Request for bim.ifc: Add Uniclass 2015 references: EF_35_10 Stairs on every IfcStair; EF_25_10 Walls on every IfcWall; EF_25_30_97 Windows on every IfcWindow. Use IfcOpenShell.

First a look at what the model holds.

```python
import ifcopenshell

model = ifcopenshell.open("bim.ifc")
print(model.schema)
print("classifications:", [c.Name for c in model.by_type("IfcClassification")])
for ifc_class in ("IfcDoor", "IfcRoof", "IfcStair", "IfcWall", "IfcWindow"):
    print(ifc_class, len(model.by_type(ifc_class)))
```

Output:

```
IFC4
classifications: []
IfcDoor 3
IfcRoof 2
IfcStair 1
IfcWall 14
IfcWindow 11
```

```python
import ifcopenshell
import ifcopenshell.api.classification

model = ifcopenshell.open("bim.ifc")

system = ifcopenshell.api.classification.add_classification(model, classification="Uniclass 2015")

codes = {
    "IfcStair": ("EF_35_10", "Stairs"),
    "IfcWall": ("EF_25_10", "Walls"),
    "IfcWindow": ("EF_25_30_97", "Windows"),
}
for ifc_class, (code, name) in codes.items():
    products = model.by_type(ifc_class)
    ifcopenshell.api.classification.add_reference(
        model, products=products, classification=system, identification=code, name=name
    )
    print(code, len(products))

model.write("bim_updated.ifc")
```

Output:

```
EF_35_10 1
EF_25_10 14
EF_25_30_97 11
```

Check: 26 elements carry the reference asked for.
